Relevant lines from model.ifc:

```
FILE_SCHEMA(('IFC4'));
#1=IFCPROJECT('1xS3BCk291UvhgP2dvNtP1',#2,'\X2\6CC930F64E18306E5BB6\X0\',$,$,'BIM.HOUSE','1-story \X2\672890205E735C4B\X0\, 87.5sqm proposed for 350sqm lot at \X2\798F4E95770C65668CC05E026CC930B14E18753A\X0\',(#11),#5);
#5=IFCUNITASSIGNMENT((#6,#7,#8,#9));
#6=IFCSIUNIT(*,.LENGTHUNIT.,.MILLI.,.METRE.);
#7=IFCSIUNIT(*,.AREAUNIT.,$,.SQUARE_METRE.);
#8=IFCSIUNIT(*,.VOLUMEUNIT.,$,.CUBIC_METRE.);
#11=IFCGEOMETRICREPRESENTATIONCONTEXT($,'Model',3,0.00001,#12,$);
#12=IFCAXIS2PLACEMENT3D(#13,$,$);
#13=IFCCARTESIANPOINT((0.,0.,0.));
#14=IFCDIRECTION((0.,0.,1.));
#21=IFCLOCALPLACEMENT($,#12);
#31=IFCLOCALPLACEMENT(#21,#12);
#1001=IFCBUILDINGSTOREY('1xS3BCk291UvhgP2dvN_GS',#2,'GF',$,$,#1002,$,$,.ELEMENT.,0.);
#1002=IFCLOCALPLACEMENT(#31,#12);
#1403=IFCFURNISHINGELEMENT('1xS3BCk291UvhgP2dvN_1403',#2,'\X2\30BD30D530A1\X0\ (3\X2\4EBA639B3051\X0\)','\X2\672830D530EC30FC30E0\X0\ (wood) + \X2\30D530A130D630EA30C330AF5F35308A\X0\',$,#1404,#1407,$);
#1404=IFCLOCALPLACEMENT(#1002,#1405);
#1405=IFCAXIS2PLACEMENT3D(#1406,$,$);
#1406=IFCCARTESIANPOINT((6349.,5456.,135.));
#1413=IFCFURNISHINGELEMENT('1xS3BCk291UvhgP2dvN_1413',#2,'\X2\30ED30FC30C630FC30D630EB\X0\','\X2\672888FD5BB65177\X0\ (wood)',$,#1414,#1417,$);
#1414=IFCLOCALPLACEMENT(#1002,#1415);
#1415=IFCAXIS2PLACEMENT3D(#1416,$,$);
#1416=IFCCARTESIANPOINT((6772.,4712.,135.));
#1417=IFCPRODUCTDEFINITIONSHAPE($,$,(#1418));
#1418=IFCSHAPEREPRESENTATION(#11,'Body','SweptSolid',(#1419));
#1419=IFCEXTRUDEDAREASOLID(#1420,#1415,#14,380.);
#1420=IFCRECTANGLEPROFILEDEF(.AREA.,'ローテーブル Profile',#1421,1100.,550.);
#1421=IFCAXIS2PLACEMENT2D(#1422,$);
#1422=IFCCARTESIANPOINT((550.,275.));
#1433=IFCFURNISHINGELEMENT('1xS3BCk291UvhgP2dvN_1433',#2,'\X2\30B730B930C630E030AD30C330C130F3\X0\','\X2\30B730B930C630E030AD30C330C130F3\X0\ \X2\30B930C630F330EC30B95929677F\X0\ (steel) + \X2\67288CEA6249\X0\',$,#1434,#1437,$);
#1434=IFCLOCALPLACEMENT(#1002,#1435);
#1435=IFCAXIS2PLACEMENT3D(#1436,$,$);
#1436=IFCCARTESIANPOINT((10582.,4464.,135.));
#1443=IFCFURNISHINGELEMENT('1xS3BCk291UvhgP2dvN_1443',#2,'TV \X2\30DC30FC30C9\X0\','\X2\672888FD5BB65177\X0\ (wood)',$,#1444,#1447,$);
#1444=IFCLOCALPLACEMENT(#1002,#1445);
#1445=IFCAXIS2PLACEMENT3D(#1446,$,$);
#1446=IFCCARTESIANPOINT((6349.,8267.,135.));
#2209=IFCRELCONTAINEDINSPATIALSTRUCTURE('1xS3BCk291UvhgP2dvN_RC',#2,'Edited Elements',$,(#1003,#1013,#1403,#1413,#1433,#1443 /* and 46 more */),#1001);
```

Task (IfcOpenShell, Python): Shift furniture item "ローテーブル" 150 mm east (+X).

```python
import ifcopenshell
import ifcopenshell.api.geometry
import ifcopenshell.util.placement
import ifcopenshell.util.unit

model = ifcopenshell.open("model.ifc")
unit_scale = ifcopenshell.util.unit.calculate_unit_scale(model)

item = model.by_id(1413)
matrix = ifcopenshell.util.placement.get_local_placement(item.ObjectPlacement)
matrix[0, 3] += 0.15 / unit_scale
ifcopenshell.api.geometry.edit_object_placement(model, product=item, matrix=matrix, is_si=False)

print(ifcopenshell.util.placement.get_local_placement(item.ObjectPlacement).round(3) + 0.0)

model.write("model-out.ifc")
```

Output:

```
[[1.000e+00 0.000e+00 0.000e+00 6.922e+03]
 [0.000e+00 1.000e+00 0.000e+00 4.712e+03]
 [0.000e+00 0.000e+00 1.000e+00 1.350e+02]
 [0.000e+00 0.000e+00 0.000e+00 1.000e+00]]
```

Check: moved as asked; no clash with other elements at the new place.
